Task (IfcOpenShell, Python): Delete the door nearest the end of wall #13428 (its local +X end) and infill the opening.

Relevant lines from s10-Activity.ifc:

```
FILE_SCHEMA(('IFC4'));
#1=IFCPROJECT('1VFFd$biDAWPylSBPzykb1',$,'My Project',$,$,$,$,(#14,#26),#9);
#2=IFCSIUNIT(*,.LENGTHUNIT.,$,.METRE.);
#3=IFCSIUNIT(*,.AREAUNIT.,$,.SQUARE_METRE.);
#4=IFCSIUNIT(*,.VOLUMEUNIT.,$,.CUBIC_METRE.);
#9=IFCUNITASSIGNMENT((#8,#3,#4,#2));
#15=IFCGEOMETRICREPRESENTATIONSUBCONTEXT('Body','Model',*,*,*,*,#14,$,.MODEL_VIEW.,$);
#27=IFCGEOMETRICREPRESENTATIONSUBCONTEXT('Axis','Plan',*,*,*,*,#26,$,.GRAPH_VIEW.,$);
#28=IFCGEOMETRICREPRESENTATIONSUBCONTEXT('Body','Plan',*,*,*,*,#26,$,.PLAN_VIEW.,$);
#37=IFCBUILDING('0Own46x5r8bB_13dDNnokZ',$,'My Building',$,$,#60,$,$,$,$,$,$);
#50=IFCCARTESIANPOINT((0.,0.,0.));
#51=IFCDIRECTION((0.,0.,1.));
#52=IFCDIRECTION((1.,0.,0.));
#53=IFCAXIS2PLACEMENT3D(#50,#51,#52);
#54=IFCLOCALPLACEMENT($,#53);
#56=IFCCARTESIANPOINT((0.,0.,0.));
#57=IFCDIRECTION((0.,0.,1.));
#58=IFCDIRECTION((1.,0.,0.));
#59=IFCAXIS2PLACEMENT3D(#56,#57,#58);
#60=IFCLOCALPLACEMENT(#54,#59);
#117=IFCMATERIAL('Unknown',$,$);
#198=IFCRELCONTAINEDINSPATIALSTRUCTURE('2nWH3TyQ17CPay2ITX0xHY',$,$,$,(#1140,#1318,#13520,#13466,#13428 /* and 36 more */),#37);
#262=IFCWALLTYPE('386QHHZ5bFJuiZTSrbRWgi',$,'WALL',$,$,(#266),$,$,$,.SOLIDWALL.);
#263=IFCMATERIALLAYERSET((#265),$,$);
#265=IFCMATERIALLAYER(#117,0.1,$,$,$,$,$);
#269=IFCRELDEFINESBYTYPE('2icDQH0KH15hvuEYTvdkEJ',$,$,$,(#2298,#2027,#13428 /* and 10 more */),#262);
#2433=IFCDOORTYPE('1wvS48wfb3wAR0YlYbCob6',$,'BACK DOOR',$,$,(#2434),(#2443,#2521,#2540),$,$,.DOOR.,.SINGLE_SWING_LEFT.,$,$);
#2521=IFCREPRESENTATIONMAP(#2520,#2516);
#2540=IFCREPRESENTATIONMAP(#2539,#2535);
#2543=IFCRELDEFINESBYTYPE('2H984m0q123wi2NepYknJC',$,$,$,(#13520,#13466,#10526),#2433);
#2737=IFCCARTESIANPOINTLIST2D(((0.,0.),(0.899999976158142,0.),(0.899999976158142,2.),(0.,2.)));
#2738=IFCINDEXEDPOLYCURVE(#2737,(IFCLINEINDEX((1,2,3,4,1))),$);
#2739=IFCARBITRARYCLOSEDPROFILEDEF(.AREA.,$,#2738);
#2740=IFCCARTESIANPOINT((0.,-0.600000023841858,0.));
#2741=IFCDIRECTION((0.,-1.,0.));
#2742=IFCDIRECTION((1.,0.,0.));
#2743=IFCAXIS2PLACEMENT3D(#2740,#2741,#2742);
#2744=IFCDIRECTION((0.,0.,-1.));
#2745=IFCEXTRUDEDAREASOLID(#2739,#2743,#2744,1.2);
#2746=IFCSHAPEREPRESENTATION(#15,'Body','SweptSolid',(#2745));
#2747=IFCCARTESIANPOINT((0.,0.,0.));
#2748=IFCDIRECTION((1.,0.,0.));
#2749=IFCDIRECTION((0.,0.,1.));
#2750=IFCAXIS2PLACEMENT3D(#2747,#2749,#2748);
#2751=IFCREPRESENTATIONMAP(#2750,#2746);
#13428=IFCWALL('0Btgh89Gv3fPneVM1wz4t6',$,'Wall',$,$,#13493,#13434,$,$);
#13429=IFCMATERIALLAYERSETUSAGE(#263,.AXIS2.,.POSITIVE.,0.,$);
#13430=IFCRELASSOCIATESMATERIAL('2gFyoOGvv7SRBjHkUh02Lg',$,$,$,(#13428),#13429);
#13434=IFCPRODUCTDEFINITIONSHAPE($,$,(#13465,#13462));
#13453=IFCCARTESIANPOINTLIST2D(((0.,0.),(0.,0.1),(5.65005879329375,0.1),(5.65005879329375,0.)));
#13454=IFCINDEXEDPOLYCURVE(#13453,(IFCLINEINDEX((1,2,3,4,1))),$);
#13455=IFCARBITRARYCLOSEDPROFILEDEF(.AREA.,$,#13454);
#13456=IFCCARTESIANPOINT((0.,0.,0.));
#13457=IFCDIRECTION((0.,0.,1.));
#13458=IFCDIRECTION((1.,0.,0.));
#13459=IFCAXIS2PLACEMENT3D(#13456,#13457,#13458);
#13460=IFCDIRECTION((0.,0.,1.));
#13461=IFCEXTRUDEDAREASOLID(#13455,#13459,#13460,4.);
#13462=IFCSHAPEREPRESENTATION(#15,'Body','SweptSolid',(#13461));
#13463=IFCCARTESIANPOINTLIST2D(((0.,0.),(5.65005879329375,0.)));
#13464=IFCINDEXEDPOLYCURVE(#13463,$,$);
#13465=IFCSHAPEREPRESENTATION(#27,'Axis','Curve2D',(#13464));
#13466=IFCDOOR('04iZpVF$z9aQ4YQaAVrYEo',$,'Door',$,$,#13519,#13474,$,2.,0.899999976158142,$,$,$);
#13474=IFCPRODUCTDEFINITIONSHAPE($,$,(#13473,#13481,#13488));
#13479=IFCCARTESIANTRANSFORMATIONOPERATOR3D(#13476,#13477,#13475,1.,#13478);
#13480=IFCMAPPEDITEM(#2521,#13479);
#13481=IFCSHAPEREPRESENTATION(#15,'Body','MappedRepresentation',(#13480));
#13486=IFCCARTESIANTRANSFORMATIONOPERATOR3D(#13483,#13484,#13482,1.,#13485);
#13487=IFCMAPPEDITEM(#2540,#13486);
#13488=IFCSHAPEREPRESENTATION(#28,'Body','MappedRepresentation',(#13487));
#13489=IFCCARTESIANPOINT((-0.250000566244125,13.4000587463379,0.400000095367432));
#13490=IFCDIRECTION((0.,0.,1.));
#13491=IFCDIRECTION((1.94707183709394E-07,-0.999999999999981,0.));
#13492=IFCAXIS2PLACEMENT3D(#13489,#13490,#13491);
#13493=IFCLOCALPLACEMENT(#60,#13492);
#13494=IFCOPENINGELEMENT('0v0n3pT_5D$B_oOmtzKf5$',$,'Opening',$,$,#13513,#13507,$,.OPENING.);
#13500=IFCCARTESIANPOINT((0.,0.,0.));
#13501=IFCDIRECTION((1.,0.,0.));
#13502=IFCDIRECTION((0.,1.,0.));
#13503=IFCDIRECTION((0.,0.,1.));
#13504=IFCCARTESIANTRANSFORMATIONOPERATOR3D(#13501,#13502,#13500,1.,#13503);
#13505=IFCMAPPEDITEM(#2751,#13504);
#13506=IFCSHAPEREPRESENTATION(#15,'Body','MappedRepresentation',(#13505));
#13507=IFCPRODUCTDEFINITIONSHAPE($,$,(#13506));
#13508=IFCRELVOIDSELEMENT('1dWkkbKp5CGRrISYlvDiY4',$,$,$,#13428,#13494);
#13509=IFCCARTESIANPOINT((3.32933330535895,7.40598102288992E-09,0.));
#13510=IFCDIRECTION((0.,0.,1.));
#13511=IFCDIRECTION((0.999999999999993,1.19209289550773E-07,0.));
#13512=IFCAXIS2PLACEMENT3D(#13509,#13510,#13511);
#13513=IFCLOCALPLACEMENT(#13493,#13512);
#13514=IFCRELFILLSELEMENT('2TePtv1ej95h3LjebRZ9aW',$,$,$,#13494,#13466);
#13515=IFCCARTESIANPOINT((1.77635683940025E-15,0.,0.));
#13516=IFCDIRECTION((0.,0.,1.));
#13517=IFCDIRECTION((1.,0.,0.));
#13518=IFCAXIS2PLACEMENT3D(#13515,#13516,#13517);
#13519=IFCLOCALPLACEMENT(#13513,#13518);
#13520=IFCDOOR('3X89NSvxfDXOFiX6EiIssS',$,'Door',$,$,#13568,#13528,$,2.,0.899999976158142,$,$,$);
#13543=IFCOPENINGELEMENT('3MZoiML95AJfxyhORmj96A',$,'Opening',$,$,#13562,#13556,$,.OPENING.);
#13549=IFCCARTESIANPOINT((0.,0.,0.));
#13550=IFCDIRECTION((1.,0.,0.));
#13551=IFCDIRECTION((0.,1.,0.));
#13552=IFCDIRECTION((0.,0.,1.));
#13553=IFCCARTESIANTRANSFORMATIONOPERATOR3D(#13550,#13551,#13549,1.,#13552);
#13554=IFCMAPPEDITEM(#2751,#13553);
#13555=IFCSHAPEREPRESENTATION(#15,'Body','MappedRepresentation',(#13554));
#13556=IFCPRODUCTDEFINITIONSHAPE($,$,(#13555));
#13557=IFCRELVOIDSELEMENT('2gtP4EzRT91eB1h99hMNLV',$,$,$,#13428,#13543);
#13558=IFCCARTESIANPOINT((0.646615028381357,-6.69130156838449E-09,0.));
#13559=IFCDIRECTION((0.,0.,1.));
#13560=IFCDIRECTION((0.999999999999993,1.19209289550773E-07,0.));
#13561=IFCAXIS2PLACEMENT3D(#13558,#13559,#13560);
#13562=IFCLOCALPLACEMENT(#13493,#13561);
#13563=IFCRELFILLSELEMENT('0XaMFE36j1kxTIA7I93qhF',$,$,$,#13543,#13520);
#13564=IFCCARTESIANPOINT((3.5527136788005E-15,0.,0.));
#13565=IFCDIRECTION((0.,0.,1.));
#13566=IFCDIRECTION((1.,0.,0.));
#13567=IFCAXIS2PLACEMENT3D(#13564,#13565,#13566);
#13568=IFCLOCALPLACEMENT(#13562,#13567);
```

```python
import ifcopenshell
import ifcopenshell.api.feature
import ifcopenshell.api.root
import ifcopenshell.geom
import ifcopenshell.util.shape

model = ifcopenshell.open("s10-Activity.ifc")
settings = ifcopenshell.geom.settings()


def volume(element):
    """Net volume in cubic metres, openings subtracted."""
    shape = ifcopenshell.geom.create_shape(settings, element)
    return ifcopenshell.util.shape.get_volume(shape.geometry)


door = model.by_guid("04iZpVF$z9aQ4YQaAVrYEo")
opening = door.FillsVoids[0].RelatingOpeningElement
wall = opening.VoidsElements[0].RelatingBuildingElement
before = volume(wall)

ifcopenshell.api.root.remove_product(model, product=door)
ifcopenshell.api.feature.remove_feature(model, feature=opening)

after = volume(wall)

print(f"wall volume {before:.3f} -> {after:.3f} m3")

model.write("s10-Activity_rev.ifc")
```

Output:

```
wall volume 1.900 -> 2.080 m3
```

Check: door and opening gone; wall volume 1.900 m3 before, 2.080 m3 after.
